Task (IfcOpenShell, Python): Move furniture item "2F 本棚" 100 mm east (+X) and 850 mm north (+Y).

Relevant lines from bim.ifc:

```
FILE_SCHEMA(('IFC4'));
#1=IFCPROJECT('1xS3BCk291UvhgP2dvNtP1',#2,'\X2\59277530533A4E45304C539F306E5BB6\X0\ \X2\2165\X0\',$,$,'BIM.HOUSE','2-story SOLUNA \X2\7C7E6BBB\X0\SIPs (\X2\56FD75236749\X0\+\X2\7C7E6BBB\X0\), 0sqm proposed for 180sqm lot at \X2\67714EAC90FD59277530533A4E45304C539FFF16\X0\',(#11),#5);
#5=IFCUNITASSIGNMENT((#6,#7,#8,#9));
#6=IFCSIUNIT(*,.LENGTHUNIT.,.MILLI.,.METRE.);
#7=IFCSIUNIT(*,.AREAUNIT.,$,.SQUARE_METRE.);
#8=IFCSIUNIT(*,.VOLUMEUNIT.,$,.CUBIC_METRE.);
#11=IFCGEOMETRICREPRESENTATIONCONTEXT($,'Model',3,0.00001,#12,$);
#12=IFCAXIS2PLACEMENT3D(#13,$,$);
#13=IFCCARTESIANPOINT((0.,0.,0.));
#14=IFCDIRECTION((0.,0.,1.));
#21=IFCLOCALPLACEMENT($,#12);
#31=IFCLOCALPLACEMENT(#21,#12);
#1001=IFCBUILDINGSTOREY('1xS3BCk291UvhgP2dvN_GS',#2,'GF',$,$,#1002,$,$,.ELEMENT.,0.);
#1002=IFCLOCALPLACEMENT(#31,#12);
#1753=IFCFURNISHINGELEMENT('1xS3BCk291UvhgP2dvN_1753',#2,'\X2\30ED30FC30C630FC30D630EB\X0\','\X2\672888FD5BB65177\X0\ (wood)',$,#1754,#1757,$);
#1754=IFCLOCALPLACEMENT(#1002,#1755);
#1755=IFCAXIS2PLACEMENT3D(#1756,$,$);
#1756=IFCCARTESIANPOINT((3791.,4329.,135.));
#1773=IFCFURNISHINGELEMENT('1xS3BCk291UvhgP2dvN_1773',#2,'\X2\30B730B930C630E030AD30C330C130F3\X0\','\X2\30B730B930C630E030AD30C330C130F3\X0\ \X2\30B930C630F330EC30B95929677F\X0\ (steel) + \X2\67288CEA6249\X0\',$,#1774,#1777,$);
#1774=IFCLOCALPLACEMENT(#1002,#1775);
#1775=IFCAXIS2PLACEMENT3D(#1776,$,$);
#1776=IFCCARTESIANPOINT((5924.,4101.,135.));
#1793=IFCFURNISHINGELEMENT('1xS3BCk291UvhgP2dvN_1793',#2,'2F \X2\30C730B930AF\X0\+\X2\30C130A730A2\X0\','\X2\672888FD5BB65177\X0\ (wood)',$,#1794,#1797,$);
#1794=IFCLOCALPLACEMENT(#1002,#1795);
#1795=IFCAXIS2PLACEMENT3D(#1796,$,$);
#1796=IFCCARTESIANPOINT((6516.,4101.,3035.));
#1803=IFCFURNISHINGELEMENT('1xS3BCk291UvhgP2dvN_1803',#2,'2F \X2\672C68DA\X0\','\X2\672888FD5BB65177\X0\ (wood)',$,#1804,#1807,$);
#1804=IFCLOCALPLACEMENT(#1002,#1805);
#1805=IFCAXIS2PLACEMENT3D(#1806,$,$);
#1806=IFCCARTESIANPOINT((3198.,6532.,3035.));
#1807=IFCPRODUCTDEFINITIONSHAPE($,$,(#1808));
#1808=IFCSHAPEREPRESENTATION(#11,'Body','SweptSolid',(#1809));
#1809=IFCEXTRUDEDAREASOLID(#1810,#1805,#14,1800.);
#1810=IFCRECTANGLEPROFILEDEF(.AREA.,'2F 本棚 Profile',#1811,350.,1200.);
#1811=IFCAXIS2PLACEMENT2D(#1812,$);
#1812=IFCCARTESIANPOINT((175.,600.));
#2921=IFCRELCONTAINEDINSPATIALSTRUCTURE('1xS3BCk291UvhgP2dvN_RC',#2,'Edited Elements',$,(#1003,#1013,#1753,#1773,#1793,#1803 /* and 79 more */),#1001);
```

```python
import ifcopenshell
import ifcopenshell.api.geometry
import ifcopenshell.util.placement

model = ifcopenshell.open("bim.ifc")

item = model.by_guid("1xS3BCk291UvhgP2dvN_1803")
matrix = ifcopenshell.util.placement.get_local_placement(item.ObjectPlacement)
matrix[0, 3] += 100.0
matrix[1, 3] += 850.0
ifcopenshell.api.geometry.edit_object_placement(model, product=item, matrix=matrix, is_si=False)

print(ifcopenshell.util.placement.get_local_placement(item.ObjectPlacement).round(3) + 0.0)

model.write("bim-out.ifc")
```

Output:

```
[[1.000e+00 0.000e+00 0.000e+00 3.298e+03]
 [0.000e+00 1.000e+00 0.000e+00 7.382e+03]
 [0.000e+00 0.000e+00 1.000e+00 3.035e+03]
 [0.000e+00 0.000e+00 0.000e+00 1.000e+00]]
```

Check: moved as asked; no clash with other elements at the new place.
